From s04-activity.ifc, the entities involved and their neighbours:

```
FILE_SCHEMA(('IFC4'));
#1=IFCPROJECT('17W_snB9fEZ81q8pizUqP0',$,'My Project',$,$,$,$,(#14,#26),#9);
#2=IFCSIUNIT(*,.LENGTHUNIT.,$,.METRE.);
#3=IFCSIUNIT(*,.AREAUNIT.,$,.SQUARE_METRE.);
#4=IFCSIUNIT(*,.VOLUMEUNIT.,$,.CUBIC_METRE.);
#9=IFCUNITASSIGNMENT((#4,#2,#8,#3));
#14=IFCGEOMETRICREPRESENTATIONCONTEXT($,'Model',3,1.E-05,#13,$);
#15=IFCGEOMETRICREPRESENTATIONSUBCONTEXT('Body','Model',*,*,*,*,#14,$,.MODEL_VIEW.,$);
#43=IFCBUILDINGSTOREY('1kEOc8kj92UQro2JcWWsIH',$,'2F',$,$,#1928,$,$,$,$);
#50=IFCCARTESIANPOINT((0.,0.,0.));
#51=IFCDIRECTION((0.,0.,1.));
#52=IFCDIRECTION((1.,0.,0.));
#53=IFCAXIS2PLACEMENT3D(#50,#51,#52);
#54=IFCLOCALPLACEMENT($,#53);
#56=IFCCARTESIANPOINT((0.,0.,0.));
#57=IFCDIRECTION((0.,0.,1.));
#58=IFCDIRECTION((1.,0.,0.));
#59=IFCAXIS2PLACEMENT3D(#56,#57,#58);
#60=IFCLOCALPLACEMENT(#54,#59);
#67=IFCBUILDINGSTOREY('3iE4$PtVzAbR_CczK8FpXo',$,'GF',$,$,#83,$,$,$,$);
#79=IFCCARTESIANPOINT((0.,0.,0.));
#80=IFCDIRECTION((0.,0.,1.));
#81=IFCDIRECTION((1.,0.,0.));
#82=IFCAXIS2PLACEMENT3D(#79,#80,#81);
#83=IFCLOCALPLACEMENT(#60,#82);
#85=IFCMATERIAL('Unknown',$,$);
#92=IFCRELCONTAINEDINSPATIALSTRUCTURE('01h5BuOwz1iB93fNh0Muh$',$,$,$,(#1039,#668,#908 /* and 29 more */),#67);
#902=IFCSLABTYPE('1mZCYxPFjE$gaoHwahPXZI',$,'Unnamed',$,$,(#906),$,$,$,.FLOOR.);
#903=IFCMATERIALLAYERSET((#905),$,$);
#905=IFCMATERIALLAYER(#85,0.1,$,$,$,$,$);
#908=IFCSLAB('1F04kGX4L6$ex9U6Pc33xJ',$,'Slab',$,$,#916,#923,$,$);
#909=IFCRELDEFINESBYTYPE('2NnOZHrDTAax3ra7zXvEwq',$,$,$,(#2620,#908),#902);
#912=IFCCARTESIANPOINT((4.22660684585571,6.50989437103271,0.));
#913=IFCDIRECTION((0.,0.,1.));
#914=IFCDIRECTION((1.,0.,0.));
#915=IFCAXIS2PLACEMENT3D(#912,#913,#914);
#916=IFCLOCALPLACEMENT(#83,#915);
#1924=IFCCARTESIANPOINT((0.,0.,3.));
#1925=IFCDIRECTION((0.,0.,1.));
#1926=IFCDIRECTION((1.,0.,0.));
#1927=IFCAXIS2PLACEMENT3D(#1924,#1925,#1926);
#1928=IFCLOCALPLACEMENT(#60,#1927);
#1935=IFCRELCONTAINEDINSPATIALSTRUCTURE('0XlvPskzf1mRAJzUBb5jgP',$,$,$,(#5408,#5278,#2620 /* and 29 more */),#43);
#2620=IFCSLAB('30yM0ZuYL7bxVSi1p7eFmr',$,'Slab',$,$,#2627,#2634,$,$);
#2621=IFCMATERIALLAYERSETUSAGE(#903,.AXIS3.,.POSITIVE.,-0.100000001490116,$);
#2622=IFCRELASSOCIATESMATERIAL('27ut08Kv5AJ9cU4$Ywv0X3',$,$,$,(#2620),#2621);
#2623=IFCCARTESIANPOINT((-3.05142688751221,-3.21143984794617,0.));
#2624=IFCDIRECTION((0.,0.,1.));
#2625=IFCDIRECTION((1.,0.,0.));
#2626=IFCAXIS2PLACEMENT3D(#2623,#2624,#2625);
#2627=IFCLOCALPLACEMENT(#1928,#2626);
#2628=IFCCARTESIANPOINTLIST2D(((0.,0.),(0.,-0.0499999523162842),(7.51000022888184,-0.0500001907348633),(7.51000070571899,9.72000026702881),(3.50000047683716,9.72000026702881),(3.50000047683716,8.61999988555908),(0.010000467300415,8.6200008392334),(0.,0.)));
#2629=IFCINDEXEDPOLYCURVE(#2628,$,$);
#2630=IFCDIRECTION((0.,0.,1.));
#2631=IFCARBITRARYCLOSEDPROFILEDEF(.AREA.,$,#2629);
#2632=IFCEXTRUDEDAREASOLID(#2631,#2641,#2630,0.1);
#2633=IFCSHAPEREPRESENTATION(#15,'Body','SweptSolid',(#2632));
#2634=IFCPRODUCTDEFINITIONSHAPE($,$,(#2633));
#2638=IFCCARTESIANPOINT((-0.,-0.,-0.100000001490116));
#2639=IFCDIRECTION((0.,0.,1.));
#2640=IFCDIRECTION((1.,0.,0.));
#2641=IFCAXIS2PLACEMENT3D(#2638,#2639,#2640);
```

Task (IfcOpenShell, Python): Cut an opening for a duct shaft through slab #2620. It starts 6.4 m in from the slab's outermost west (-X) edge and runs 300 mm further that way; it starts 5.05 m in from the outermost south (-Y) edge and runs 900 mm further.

```python
import numpy as np
import ifcopenshell
import ifcopenshell.api.feature
import ifcopenshell.api.geometry
import ifcopenshell.api.root
import ifcopenshell.geom
import ifcopenshell.util.placement
import ifcopenshell.util.representation
import ifcopenshell.util.shape
import ifcopenshell.util.unit

model = ifcopenshell.open("s04-activity.ifc")
unit_scale = ifcopenshell.util.unit.calculate_unit_scale(model)
settings = ifcopenshell.geom.settings()


def volume(element):
    """Net volume in cubic metres, openings subtracted."""
    shape = ifcopenshell.geom.create_shape(settings, element)
    return ifcopenshell.util.shape.get_volume(shape.geometry)


slab = model.by_guid("30yM0ZuYL7bxVSi1p7eFmr")
before = volume(slab)

# Extent in the slab's own axes, in metres. The edges named are its -X and -Y sides.
slab_shape = ifcopenshell.geom.create_shape(settings, slab)
vertices = ifcopenshell.util.shape.get_vertices(slab_shape.geometry)
x_min, y_min, bottom = vertices.min(axis=0)
top = vertices[:, 2].max()

opening = ifcopenshell.api.root.create_entity(model, ifc_class="IfcOpeningElement", name="Duct shaft opening", predefined_type="OPENING")
context = ifcopenshell.util.representation.get_context(model, "Model", "Body", "MODEL_VIEW")
width, depth = 0.3, 0.9
outline = [(0.0, 0.0), (width, 0.0), (width, depth), (0.0, depth), (0.0, 0.0)]
# Overshoot both faces by 50 mm so the cut is clean.
shape = ifcopenshell.api.geometry.add_slab_representation(
    model, context=context, depth=top - bottom + 0.1, polyline=outline
)
ifcopenshell.api.geometry.assign_representation(model, product=opening, representation=shape)

matrix = ifcopenshell.util.placement.get_local_placement(slab.ObjectPlacement)
matrix[:, 3] = matrix @ np.append(np.array([x_min + 6.4, y_min + 5.05, bottom - 0.05]) / unit_scale, 1.0)
ifcopenshell.api.geometry.edit_object_placement(model, product=opening, matrix=matrix, is_si=False)
ifcopenshell.api.feature.add_feature(model, feature=opening, element=slab)

after = volume(slab)

print(f"slab volume {before:.3f} -> {after:.3f} m3")

model.write("s04-activity-out.ifc")
```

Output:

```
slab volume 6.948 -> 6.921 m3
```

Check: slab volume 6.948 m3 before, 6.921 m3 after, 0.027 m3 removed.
